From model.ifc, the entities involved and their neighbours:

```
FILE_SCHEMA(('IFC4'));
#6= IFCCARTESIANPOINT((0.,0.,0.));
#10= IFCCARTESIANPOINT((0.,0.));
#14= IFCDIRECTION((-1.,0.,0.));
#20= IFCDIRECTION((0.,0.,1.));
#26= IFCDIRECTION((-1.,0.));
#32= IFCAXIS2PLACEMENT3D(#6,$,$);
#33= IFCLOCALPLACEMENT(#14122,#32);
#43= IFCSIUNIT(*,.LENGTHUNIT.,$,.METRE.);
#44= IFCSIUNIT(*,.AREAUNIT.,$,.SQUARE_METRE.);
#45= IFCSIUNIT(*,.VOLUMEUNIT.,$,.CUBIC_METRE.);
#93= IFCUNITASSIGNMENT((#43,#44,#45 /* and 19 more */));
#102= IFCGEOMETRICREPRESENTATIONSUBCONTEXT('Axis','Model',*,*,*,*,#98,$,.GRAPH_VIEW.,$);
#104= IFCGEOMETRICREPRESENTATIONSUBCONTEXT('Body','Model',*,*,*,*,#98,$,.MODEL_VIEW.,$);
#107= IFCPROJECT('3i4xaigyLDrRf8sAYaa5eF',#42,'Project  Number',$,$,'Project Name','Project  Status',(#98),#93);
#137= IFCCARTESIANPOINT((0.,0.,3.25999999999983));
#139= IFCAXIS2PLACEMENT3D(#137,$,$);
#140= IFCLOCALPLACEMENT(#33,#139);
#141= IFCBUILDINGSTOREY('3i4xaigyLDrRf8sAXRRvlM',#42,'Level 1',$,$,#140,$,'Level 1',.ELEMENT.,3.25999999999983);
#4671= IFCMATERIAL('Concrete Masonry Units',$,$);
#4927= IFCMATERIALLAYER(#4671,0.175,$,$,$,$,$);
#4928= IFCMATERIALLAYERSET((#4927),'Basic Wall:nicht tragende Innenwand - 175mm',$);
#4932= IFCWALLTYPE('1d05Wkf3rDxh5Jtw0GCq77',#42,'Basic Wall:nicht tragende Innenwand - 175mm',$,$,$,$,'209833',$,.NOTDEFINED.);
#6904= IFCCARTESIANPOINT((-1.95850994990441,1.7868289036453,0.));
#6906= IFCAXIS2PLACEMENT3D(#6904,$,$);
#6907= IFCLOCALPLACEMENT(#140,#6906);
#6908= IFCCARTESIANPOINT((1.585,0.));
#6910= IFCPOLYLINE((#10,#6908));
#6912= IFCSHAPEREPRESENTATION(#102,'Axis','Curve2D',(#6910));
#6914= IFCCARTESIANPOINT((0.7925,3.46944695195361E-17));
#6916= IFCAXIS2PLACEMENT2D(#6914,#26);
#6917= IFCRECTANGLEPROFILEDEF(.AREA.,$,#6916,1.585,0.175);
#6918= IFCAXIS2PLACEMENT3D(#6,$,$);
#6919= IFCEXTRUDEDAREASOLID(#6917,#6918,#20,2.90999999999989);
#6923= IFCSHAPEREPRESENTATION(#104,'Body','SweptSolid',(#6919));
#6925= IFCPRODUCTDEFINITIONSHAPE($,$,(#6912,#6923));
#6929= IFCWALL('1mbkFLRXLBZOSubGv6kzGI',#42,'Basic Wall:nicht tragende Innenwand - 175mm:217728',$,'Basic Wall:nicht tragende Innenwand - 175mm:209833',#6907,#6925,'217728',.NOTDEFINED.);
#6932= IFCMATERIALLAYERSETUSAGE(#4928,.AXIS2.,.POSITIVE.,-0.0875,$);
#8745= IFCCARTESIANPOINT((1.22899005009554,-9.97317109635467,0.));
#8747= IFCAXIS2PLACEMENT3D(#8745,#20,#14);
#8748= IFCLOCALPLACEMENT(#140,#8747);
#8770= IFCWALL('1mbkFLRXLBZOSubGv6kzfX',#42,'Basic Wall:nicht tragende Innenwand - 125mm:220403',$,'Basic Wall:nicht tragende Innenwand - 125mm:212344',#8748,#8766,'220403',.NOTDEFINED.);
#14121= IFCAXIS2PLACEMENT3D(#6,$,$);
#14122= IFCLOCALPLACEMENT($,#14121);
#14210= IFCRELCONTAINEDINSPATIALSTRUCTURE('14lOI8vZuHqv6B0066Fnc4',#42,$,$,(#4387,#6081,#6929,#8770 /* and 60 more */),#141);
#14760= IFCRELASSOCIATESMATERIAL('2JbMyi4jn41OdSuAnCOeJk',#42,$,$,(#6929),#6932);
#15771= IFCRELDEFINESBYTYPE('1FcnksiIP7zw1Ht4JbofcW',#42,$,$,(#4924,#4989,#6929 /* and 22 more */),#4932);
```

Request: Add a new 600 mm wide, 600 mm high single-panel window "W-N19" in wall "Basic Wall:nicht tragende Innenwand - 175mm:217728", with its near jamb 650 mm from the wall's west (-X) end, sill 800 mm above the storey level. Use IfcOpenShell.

```python
import numpy as np
import ifcopenshell
import ifcopenshell.api.feature
import ifcopenshell.api.geometry
import ifcopenshell.api.root
import ifcopenshell.api.spatial
import ifcopenshell.geom
import ifcopenshell.util.element
import ifcopenshell.util.placement
import ifcopenshell.util.representation
import ifcopenshell.util.shape
import ifcopenshell.util.unit

model = ifcopenshell.open("model.ifc")
unit_scale = ifcopenshell.util.unit.calculate_unit_scale(model)
settings = ifcopenshell.geom.settings()


def volume(element):
    """Net volume in cubic metres, openings subtracted."""
    shape = ifcopenshell.geom.create_shape(settings, element)
    return ifcopenshell.util.shape.get_volume(shape.geometry)


wall = model.by_guid("1mbkFLRXLBZOSubGv6kzGI")
storey = ifcopenshell.util.element.get_container(wall, ifc_class="IfcBuildingStorey")
context = ifcopenshell.util.representation.get_context(model, "Model", "Body", "MODEL_VIEW")
before = volume(wall)

width, height, from_end, sill = 0.6, 0.6, 0.65, 0.8  # metres

# The wall runs along its own X axis, and the end named is its -X end.
wall_shape = ifcopenshell.geom.create_shape(settings, wall)
x, y, z = ifcopenshell.util.shape.get_vertices(wall_shape.geometry).T
start = x.min() + from_end
face, thickness = float(y.min()), float(y.max() - y.min())
wall_matrix = ifcopenshell.util.placement.get_local_placement(wall.ObjectPlacement)
level = ifcopenshell.util.placement.get_local_placement(storey.ObjectPlacement)[2, 3]


def in_wall(x, y):
    """Placement at x, y metres in the wall's axes, at sill height."""
    matrix = wall_matrix.copy()
    matrix[:, 3] = wall_matrix @ np.array([x / unit_scale, y / unit_scale, 0.0, 1.0])
    matrix[2, 3] = level + sill / unit_scale
    return matrix


# Opening: a box that overshoots both wall faces by 50 mm.
opening = ifcopenshell.api.root.create_entity(model, ifc_class="IfcOpeningElement", predefined_type="OPENING")
box = ifcopenshell.api.geometry.add_wall_representation(
    model, context=context, length=width, height=height, thickness=thickness + 0.1
)
ifcopenshell.api.geometry.assign_representation(model, product=opening, representation=box)
ifcopenshell.api.geometry.edit_object_placement(model, product=opening, matrix=in_wall(start, face - 0.05), is_si=False)
ifcopenshell.api.feature.add_feature(model, feature=opening, element=wall)

window = ifcopenshell.api.root.create_entity(model, ifc_class="IfcWindow", name="W-N19", predefined_type="WINDOW")
window.OverallWidth, window.OverallHeight = width / unit_scale, height / unit_scale
window.PartitioningType = "SINGLE_PANEL"
body = ifcopenshell.api.geometry.add_window_representation(
    model,
    context=context,
    overall_width=window.OverallWidth,
    overall_height=window.OverallHeight,
    partition_type="SINGLE_PANEL",
)
ifcopenshell.api.geometry.assign_representation(model, product=window, representation=body)
ifcopenshell.api.spatial.assign_container(model, products=[window], relating_structure=storey)
ifcopenshell.api.feature.add_filling(model, opening=opening, element=window)

# Centre the window in the wall's thickness.
ifcopenshell.api.geometry.edit_object_placement(model, product=window, matrix=in_wall(start, face), is_si=False)
window_shape = ifcopenshell.geom.create_shape(settings, window)
depth = ifcopenshell.util.shape.get_vertices(window_shape.geometry)[:, 1]
offset = face + thickness / 2 - (depth.min() + depth.max()) / 2
ifcopenshell.api.geometry.edit_object_placement(model, product=window, matrix=in_wall(start, offset), is_si=False)

after = volume(wall)

print(f"wall volume {before:.3f} -> {after:.3f} m3")

model.write("model_rev.ifc")
```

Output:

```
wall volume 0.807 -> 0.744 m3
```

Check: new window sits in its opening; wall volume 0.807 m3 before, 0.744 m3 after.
